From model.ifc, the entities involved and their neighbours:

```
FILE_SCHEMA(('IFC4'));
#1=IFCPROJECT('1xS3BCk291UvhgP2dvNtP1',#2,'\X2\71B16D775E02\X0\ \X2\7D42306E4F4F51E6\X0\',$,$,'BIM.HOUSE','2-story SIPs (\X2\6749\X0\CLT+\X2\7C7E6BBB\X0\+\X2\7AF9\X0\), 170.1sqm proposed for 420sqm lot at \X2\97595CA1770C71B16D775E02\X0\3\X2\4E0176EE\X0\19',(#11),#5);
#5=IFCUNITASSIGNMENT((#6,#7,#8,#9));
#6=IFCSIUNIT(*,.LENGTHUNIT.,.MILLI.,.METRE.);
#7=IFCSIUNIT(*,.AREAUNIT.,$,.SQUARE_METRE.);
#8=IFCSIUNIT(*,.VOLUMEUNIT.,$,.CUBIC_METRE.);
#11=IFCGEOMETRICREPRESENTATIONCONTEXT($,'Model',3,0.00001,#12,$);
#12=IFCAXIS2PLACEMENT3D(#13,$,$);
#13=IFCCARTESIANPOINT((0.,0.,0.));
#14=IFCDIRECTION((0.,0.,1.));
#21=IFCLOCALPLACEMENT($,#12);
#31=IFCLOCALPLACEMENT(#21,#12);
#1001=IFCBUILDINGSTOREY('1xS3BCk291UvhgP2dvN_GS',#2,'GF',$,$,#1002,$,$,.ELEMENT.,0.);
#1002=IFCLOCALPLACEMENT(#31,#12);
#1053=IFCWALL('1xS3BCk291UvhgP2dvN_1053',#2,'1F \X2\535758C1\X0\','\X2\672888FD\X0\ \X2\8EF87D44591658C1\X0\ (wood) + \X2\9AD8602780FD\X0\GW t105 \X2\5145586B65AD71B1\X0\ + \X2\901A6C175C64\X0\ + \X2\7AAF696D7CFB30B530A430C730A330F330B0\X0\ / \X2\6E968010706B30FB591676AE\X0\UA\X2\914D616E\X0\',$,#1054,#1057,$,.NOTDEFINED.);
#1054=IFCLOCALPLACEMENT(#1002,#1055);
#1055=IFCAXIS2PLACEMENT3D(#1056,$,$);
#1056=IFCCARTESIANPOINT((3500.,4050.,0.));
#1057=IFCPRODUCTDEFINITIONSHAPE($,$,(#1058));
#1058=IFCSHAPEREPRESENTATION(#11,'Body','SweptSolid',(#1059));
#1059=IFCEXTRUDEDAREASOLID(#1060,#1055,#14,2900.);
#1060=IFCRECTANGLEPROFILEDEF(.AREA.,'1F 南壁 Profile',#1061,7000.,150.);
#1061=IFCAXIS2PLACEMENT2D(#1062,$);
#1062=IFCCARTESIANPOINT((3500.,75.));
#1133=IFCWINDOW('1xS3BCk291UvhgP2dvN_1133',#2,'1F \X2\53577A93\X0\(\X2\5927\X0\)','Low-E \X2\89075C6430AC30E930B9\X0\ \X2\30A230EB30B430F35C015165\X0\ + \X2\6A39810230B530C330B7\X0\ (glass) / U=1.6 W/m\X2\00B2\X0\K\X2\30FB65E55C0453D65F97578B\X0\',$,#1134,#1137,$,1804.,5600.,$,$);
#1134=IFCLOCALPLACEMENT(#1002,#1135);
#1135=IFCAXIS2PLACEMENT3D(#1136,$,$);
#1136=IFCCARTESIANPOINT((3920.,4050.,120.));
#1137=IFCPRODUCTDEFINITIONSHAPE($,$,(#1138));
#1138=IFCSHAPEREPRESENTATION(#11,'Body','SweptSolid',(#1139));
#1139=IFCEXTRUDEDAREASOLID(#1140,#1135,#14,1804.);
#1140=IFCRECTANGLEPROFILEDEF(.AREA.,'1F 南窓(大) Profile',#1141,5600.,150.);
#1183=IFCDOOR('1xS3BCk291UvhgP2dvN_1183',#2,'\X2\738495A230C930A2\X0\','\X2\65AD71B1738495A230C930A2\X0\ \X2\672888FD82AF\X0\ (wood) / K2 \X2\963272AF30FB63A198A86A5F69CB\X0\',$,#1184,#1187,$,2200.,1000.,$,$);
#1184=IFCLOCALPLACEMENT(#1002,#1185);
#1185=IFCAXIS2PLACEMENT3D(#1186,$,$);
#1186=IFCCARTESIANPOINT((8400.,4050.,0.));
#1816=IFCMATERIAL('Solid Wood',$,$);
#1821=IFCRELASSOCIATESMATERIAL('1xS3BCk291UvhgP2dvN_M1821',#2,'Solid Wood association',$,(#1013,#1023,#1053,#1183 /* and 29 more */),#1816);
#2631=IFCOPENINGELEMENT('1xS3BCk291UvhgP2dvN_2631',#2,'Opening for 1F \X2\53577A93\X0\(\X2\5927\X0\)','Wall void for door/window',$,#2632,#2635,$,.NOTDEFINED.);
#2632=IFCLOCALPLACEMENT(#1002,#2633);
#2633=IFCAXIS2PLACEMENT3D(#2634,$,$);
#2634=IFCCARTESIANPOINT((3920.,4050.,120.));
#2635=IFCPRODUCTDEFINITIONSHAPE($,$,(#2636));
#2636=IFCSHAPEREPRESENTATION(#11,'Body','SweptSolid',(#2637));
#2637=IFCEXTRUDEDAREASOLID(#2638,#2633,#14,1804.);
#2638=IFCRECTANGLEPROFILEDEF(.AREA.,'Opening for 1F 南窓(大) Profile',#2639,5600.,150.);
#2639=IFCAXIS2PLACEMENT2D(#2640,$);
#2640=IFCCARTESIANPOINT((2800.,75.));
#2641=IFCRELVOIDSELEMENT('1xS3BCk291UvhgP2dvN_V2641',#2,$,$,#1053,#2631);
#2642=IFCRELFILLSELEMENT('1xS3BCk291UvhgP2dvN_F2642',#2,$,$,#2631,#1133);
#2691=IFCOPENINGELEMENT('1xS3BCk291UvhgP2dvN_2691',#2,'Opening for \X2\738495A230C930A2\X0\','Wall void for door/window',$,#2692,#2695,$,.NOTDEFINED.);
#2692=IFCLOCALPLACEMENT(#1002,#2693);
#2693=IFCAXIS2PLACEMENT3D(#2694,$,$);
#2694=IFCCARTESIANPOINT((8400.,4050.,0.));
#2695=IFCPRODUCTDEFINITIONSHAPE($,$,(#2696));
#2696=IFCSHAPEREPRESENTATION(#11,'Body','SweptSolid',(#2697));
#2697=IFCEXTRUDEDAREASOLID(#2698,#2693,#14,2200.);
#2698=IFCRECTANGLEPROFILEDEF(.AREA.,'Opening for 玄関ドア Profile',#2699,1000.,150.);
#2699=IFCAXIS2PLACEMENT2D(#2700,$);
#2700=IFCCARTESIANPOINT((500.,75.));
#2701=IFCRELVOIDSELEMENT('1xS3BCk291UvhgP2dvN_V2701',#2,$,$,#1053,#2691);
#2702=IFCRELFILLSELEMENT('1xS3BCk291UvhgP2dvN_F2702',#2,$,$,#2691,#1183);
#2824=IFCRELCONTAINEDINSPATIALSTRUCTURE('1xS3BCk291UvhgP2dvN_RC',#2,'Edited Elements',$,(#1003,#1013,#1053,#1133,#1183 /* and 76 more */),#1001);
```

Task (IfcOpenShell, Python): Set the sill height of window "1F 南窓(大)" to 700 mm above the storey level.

```python
import numpy as np
import ifcopenshell
import ifcopenshell.api.geometry
import ifcopenshell.geom
import ifcopenshell.util.element
import ifcopenshell.util.placement
import ifcopenshell.util.shape
import ifcopenshell.util.unit

model = ifcopenshell.open("model.ifc")
unit_scale = ifcopenshell.util.unit.calculate_unit_scale(model)

window = model.by_guid("1xS3BCk291UvhgP2dvN_1133")
opening = window.FillsVoids[0].RelatingOpeningElement
storey = ifcopenshell.util.element.get_container(window, ifc_class="IfcBuildingStorey")
level = ifcopenshell.util.placement.get_local_placement(storey.ObjectPlacement)[2, 3]

# The opening's origin need not be at the sill, so measure its lowest point.
shape = ifcopenshell.geom.create_shape(ifcopenshell.geom.settings(), opening)
bottom = ifcopenshell.util.shape.get_shape_bottom_elevation(shape, shape.geometry) / unit_scale
dz = level + 0.7 / unit_scale - bottom

shift = np.array([0.0, 0.0, dz])
# The window is not placed relative to its opening, so move both.
for product in (opening, window):
    matrix = ifcopenshell.util.placement.get_local_placement(product.ObjectPlacement)
    matrix[:3, 3] += shift
    ifcopenshell.api.geometry.edit_object_placement(model, product=product, matrix=matrix, is_si=False)

print(f"moved by {dz * unit_scale:+.3f} m")

model.write("model_updated.ifc")
```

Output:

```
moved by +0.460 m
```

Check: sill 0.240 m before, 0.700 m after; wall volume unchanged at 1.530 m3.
